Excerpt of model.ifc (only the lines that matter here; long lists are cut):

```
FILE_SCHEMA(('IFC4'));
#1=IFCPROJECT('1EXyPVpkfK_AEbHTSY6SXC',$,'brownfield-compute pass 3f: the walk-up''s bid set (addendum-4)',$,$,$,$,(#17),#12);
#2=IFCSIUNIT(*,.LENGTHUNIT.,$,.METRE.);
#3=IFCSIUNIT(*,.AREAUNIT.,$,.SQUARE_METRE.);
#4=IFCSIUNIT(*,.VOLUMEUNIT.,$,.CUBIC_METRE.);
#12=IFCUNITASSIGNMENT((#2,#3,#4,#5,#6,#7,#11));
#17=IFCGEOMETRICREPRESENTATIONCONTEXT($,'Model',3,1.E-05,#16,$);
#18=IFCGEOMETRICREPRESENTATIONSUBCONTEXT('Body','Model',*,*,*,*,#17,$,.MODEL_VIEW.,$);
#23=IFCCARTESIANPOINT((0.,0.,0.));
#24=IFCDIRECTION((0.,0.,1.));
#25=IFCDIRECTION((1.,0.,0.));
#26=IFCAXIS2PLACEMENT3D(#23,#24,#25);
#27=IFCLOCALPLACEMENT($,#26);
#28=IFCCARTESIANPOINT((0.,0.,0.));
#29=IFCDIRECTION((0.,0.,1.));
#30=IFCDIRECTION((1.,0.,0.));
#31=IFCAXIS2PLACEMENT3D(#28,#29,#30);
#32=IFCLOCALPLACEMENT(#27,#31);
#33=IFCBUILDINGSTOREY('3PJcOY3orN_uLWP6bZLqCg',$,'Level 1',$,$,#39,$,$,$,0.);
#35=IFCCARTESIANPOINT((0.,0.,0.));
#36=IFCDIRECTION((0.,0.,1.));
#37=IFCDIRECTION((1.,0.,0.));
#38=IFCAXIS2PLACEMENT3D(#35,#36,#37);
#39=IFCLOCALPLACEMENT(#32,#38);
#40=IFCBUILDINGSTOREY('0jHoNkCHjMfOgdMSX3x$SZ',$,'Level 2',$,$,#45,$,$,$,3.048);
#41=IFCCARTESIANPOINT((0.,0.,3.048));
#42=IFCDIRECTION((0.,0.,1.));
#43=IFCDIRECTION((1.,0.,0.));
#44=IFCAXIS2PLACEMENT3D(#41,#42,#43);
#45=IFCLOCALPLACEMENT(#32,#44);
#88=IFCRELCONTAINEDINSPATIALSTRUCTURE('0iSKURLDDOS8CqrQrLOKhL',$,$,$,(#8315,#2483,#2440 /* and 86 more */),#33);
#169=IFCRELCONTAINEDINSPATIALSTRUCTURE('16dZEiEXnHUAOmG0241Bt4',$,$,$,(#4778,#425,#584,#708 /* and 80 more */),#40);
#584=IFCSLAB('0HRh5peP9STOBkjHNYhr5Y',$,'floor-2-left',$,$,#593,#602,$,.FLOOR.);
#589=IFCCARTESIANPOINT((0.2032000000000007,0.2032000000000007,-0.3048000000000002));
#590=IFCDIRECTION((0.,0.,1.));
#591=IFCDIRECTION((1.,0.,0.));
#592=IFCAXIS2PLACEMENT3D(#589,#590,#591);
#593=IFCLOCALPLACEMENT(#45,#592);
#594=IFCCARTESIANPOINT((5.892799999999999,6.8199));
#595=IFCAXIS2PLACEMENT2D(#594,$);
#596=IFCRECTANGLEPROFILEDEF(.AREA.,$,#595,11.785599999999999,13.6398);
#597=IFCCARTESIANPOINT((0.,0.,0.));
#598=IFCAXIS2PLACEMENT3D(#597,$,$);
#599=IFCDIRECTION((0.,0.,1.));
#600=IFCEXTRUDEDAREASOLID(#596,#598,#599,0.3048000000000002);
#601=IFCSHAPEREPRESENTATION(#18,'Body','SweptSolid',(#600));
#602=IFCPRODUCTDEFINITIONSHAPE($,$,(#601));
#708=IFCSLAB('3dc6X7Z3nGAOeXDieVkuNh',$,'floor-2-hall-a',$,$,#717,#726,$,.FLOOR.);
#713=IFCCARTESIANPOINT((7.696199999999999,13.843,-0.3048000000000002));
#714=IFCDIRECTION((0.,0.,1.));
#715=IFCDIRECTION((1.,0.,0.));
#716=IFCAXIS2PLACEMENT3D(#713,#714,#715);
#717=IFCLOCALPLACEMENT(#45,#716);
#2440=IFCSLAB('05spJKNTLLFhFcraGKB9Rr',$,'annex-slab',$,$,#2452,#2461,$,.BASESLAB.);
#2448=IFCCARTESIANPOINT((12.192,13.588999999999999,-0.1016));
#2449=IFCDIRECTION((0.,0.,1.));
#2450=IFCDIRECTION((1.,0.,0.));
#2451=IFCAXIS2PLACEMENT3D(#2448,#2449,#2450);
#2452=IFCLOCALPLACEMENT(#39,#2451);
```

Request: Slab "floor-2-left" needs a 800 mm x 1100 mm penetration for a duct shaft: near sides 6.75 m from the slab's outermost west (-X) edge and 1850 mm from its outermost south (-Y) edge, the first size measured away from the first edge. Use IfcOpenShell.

```python
import numpy as np
import ifcopenshell
import ifcopenshell.api.feature
import ifcopenshell.api.geometry
import ifcopenshell.api.root
import ifcopenshell.geom
import ifcopenshell.util.placement
import ifcopenshell.util.representation
import ifcopenshell.util.shape
import ifcopenshell.util.unit

model = ifcopenshell.open("model.ifc")
unit_scale = ifcopenshell.util.unit.calculate_unit_scale(model)
settings = ifcopenshell.geom.settings()


def volume(element):
    """Net volume in cubic metres, openings subtracted."""
    shape = ifcopenshell.geom.create_shape(settings, element)
    return ifcopenshell.util.shape.get_volume(shape.geometry)


slab = model.by_id(584)
before = volume(slab)

# Extent in the slab's own axes, in metres. The edges named are its -X and -Y sides.
slab_shape = ifcopenshell.geom.create_shape(settings, slab)
vertices = ifcopenshell.util.shape.get_vertices(slab_shape.geometry)
x_min, y_min, bottom = vertices.min(axis=0)
top = vertices[:, 2].max()

opening = ifcopenshell.api.root.create_entity(model, ifc_class="IfcOpeningElement", name="Duct shaft opening", predefined_type="OPENING")
context = ifcopenshell.util.representation.get_context(model, "Model", "Body", "MODEL_VIEW")
width, depth = 0.8, 1.1
outline = [(0.0, 0.0), (width, 0.0), (width, depth), (0.0, depth), (0.0, 0.0)]
# Overshoot both faces by 50 mm so the cut is clean.
shape = ifcopenshell.api.geometry.add_slab_representation(
    model, context=context, depth=top - bottom + 0.1, polyline=outline
)
ifcopenshell.api.geometry.assign_representation(model, product=opening, representation=shape)

matrix = ifcopenshell.util.placement.get_local_placement(slab.ObjectPlacement)
matrix[:, 3] = matrix @ np.append(np.array([x_min + 6.75, y_min + 1.85, bottom - 0.05]) / unit_scale, 1.0)
ifcopenshell.api.geometry.edit_object_placement(model, product=opening, matrix=matrix, is_si=False)
ifcopenshell.api.feature.add_feature(model, feature=opening, element=slab)

after = volume(slab)

print(f"slab volume {before:.3f} -> {after:.3f} m3")

model.write("model-out.ifc")
```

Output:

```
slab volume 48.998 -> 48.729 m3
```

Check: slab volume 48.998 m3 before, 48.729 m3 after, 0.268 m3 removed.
